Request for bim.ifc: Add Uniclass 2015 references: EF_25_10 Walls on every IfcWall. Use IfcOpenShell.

First a look at what the model holds.

```python
import ifcopenshell

model = ifcopenshell.open("bim.ifc")
print(model.schema)
print("classifications:", [c.Name for c in model.by_type("IfcClassification")])
for ifc_class in ("IfcDoor", "IfcRoof", "IfcStair", "IfcWall", "IfcWindow"):
    print(ifc_class, len(model.by_type(ifc_class)))
```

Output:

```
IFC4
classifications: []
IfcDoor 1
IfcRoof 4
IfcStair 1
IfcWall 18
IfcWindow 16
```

```python
import ifcopenshell
import ifcopenshell.api.classification

model = ifcopenshell.open("bim.ifc")

system = ifcopenshell.api.classification.add_classification(model, classification="Uniclass 2015")

codes = {
    "IfcWall": ("EF_25_10", "Walls"),
}
for ifc_class, (code, name) in codes.items():
    products = model.by_type(ifc_class)
    ifcopenshell.api.classification.add_reference(
        model, products=products, classification=system, identification=code, name=name
    )
    print(code, len(products))

model.write("bim_rev.ifc")
```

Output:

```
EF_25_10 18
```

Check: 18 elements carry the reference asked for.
